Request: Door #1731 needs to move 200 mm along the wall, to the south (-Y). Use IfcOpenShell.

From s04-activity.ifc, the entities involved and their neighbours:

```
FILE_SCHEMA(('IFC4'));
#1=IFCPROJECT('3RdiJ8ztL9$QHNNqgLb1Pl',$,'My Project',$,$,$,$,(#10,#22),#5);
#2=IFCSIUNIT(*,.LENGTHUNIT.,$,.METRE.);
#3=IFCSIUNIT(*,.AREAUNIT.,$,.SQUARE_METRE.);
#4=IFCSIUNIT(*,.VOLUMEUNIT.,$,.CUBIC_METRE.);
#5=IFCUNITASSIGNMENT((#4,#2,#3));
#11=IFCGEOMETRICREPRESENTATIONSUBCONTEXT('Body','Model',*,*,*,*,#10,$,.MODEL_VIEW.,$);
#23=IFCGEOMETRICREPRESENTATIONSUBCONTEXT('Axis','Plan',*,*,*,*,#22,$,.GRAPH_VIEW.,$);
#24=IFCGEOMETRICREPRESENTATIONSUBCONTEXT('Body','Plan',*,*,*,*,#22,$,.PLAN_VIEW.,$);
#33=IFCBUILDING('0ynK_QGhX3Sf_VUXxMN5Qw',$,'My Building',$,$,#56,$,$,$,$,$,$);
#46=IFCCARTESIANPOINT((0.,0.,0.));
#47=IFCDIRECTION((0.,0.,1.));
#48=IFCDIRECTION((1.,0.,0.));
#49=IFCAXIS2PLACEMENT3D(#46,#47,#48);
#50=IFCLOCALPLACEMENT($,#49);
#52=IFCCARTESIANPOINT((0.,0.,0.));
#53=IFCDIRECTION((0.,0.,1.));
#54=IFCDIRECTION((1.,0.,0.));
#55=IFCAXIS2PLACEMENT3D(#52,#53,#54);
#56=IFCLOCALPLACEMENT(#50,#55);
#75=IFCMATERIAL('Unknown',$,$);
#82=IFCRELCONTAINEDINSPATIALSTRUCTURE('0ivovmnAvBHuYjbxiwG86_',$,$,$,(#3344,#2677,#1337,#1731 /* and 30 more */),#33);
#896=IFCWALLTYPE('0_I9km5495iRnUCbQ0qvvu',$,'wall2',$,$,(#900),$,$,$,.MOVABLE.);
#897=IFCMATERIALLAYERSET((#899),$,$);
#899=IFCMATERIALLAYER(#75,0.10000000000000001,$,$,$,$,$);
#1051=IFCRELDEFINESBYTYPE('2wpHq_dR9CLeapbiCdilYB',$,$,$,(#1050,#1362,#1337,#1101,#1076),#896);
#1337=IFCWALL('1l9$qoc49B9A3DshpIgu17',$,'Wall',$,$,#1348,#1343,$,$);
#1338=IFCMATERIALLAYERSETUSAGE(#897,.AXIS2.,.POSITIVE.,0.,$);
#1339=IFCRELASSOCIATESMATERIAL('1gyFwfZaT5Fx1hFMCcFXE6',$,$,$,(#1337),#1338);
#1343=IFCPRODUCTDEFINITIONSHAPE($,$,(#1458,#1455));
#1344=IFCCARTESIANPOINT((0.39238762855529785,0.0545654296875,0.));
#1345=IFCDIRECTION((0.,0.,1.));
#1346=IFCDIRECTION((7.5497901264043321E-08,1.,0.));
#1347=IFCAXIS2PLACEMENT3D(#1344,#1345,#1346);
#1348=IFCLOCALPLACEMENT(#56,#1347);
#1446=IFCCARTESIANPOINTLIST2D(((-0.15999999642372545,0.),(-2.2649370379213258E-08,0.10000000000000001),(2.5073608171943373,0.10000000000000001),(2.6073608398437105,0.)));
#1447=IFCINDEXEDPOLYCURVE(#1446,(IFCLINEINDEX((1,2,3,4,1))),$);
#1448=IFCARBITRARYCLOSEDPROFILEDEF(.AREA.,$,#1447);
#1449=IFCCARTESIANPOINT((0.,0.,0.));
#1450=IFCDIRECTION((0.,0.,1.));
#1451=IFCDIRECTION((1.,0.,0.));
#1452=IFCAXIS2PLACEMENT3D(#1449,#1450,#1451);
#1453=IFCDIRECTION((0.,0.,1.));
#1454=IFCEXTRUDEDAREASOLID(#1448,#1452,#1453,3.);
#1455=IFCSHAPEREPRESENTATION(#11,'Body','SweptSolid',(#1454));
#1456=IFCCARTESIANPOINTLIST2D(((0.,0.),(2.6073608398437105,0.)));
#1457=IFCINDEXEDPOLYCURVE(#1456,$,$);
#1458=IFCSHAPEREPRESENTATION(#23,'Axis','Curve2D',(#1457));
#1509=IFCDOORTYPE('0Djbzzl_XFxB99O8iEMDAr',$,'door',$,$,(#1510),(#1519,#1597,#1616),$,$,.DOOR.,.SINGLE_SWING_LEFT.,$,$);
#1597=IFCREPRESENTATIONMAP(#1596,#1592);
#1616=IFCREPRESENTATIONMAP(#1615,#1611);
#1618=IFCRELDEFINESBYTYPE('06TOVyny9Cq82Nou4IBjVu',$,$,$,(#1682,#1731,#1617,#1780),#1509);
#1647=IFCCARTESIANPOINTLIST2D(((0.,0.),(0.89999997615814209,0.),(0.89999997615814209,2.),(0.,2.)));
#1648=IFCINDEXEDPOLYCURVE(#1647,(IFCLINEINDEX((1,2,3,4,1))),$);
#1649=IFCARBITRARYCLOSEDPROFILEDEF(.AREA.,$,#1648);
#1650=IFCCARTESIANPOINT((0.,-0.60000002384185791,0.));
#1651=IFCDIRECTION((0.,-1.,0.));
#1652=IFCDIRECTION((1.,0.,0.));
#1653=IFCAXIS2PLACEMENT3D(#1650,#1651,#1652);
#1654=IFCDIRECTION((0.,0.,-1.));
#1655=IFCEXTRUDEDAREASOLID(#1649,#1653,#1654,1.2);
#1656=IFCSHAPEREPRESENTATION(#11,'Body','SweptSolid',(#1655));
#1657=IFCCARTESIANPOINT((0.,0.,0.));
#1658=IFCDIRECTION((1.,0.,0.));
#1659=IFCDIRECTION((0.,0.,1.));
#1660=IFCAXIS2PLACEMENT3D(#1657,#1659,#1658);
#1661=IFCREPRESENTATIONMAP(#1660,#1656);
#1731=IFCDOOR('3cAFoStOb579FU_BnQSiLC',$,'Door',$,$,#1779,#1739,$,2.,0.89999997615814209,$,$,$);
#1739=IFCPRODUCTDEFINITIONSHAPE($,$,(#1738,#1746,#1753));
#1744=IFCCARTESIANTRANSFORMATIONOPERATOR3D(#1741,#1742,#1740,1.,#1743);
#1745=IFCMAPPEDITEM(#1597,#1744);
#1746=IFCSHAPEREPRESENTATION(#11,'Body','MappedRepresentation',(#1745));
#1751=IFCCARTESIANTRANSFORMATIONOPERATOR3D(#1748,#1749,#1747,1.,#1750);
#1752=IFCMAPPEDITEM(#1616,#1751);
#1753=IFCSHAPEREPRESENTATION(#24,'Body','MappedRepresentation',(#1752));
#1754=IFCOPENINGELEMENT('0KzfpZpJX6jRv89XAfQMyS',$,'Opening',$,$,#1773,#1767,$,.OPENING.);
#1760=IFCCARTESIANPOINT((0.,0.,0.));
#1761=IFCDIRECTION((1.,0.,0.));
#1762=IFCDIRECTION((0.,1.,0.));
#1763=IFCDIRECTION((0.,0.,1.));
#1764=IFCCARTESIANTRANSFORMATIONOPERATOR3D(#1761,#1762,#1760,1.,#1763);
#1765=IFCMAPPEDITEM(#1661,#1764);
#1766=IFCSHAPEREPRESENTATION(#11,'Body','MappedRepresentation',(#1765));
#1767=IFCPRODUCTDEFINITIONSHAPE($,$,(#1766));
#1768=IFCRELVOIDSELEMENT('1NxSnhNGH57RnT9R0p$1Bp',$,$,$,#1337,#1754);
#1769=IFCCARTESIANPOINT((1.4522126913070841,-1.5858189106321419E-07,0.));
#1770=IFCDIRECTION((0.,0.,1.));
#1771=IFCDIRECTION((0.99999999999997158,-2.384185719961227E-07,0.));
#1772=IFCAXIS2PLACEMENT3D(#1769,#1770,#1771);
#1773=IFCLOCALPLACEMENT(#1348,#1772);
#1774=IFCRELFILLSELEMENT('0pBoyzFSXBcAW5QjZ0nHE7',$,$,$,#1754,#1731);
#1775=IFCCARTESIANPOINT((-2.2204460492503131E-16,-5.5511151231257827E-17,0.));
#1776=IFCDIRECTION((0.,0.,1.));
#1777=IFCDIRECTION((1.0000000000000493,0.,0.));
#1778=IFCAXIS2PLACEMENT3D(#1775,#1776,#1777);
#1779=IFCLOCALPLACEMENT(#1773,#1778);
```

```python
import ifcopenshell
import ifcopenshell.api.geometry
import ifcopenshell.util.placement
import ifcopenshell.util.unit

model = ifcopenshell.open("s04-activity.ifc")
unit_scale = ifcopenshell.util.unit.calculate_unit_scale(model)

door = model.by_guid("3cAFoStOb579FU_BnQSiLC")
opening = door.FillsVoids[0].RelatingOpeningElement
wall = opening.VoidsElements[0].RelatingBuildingElement

wall_matrix = ifcopenshell.util.placement.get_local_placement(wall.ObjectPlacement)
shift = wall_matrix[:3, 0] * -0.2 / unit_scale
before = ifcopenshell.util.placement.get_local_placement(door.ObjectPlacement)[:3, 3].copy()

# The door is placed relative to its opening, so it follows when the opening moves.
matrix = ifcopenshell.util.placement.get_local_placement(opening.ObjectPlacement)
matrix[:3, 3] += shift
ifcopenshell.api.geometry.edit_object_placement(
    model, product=opening, matrix=matrix, is_si=False, should_transform_children=True
)

after = ifcopenshell.util.placement.get_local_placement(door.ObjectPlacement)[:3, 3]
print("door moved by", (after - before).round(3) + 0.0)

model.write("s04-activity_rev.ifc")
```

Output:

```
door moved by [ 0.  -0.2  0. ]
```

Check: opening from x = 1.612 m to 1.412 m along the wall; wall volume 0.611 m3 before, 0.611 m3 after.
